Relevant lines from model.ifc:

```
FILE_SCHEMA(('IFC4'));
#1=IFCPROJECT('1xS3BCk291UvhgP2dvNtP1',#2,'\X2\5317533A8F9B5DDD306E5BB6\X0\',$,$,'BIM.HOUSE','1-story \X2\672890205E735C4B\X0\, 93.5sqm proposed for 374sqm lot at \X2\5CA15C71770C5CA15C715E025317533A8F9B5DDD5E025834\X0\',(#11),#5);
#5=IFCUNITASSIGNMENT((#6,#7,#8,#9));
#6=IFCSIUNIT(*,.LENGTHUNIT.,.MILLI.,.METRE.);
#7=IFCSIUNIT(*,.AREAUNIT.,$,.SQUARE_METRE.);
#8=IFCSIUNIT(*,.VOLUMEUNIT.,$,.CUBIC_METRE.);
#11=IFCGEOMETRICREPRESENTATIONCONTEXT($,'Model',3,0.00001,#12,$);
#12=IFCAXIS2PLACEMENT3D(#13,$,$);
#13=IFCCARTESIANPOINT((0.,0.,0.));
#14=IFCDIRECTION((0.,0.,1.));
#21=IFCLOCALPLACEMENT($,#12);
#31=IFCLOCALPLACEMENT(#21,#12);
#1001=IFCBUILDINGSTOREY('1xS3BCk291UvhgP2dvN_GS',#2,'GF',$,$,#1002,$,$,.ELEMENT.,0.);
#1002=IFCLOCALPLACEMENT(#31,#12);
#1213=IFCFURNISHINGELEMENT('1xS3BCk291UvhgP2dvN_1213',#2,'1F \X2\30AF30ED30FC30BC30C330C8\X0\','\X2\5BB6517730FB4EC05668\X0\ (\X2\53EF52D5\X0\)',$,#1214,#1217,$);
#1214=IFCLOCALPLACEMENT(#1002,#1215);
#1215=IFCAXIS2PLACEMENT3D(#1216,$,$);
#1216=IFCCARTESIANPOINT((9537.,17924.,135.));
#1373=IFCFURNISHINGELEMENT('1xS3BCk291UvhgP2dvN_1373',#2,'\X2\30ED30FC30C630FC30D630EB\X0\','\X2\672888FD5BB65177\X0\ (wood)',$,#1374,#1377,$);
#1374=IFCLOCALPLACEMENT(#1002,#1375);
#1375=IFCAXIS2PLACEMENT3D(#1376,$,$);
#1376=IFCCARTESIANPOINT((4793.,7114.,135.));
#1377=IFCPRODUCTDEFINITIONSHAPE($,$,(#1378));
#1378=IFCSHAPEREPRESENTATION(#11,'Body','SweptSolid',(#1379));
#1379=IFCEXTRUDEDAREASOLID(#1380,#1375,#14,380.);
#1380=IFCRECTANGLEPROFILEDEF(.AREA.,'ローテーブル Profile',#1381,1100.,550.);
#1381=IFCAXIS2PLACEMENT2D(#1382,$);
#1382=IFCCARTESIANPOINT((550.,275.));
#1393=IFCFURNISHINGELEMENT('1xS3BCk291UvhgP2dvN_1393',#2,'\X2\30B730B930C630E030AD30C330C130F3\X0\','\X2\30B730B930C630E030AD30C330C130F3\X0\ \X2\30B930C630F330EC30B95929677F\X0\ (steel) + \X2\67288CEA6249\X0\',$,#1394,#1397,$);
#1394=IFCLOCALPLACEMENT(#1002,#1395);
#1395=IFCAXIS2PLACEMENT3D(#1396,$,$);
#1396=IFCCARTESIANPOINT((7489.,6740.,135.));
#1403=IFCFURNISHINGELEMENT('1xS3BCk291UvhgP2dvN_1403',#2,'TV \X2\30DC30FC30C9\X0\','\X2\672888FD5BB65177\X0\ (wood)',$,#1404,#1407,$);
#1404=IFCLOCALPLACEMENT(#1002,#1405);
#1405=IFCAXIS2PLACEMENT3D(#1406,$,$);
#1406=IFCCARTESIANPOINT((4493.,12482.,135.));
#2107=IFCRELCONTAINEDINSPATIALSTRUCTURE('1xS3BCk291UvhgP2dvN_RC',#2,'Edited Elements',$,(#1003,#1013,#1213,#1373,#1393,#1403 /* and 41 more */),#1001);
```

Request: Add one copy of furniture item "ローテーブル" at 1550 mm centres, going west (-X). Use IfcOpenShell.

```python
import numpy as np
import ifcopenshell
import ifcopenshell.api.geometry
import ifcopenshell.api.root
import ifcopenshell.util.element
import ifcopenshell.util.placement

model = ifcopenshell.open("model.ifc")


def reuse_history(source, copy):
    """copy_class also copies each property set's owner history, people and application; keep the originals."""
    for rel in copy.IsDefinedBy:
        if rel.is_a("IfcRelDefinesByProperties") and (history := rel.RelatingPropertyDefinition.OwnerHistory):
            rel.RelatingPropertyDefinition.OwnerHistory = source.OwnerHistory
            ifcopenshell.util.element.remove_deep2(model, history)


source = model.by_id(1373)
base = ifcopenshell.util.placement.get_local_placement(source.ObjectPlacement)
step = np.array([-1.0, 0.0, 0.0]) * 1550.0

for i in range(1, 2):
    copy = ifcopenshell.api.root.copy_class(model, product=source)
    copy.Representation = ifcopenshell.util.element.copy_deep(
        model, source.Representation, exclude=["IfcGeometricRepresentationContext", "IfcRepresentationMap"]
    )
    reuse_history(source, copy)
    matrix = base.copy()
    matrix[:3, 3] += i * step
    print("added at", matrix[:3, 3].round(3) + 0.0)
    ifcopenshell.api.geometry.edit_object_placement(model, product=copy, matrix=matrix, is_si=False)

model.write("model_updated.ifc")
```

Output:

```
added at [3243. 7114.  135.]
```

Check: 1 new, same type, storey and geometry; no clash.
